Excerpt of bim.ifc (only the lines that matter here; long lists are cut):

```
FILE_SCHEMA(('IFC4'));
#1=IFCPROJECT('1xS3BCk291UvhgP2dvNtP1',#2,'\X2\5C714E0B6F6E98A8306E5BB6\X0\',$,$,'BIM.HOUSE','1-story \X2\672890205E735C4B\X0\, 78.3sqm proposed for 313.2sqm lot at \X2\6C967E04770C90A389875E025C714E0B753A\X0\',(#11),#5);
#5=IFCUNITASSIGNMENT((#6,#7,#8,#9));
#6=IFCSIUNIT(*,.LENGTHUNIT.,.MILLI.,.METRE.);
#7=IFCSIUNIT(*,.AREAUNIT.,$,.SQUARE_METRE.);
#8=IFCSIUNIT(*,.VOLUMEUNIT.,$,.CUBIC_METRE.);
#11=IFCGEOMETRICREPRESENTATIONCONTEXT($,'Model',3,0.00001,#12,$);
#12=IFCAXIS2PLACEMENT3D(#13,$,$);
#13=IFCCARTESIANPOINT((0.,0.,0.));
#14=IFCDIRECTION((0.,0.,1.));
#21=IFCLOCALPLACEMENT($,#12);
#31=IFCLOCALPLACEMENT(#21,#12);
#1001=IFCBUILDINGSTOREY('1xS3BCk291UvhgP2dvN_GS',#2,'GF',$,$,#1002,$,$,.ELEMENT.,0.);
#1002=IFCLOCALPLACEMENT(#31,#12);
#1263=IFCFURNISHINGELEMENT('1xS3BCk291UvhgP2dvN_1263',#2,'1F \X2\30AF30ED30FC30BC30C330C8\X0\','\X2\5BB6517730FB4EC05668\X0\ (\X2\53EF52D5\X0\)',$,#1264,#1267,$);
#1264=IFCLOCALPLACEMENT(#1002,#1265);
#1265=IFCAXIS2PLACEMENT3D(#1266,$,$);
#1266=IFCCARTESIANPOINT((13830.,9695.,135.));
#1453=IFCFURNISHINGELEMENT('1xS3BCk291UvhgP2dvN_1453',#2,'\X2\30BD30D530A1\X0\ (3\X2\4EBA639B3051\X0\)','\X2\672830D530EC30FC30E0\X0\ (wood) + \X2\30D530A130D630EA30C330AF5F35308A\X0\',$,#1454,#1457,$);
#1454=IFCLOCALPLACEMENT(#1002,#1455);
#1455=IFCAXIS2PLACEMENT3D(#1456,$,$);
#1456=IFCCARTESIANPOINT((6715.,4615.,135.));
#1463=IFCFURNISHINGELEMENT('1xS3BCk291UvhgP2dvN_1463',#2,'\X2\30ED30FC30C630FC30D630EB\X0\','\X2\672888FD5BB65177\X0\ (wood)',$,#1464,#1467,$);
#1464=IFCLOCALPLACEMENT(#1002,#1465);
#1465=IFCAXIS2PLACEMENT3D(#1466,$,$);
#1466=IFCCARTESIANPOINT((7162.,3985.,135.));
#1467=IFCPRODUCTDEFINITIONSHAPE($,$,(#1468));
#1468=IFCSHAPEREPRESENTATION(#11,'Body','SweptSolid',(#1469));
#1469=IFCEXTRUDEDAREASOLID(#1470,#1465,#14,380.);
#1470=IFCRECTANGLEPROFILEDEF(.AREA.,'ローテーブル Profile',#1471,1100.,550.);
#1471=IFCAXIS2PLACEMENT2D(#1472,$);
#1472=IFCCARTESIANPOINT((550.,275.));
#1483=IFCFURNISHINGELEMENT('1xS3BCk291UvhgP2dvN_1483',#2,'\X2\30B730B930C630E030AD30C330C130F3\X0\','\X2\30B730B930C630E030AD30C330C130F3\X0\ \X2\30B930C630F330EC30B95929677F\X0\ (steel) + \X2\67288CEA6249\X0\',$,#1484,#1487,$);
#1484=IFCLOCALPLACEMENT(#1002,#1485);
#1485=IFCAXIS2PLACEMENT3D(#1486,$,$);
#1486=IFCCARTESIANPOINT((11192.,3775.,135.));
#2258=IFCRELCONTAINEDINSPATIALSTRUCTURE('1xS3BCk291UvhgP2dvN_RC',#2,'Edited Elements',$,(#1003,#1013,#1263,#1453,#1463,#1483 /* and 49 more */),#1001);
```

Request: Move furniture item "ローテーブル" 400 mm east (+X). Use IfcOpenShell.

```python
import ifcopenshell
import ifcopenshell.api.geometry
import ifcopenshell.util.placement
import ifcopenshell.util.unit

model = ifcopenshell.open("bim.ifc")
unit_scale = ifcopenshell.util.unit.calculate_unit_scale(model)

item = model.by_guid("1xS3BCk291UvhgP2dvN_1463")
matrix = ifcopenshell.util.placement.get_local_placement(item.ObjectPlacement)
matrix[0, 3] += 0.4 / unit_scale
ifcopenshell.api.geometry.edit_object_placement(model, product=item, matrix=matrix, is_si=False)

print(ifcopenshell.util.placement.get_local_placement(item.ObjectPlacement).round(3) + 0.0)

model.write("bim_updated.ifc")
```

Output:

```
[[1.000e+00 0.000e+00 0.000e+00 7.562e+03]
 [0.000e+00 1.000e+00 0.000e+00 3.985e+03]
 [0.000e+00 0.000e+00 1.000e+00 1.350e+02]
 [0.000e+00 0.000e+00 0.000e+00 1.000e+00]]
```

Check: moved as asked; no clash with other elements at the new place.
